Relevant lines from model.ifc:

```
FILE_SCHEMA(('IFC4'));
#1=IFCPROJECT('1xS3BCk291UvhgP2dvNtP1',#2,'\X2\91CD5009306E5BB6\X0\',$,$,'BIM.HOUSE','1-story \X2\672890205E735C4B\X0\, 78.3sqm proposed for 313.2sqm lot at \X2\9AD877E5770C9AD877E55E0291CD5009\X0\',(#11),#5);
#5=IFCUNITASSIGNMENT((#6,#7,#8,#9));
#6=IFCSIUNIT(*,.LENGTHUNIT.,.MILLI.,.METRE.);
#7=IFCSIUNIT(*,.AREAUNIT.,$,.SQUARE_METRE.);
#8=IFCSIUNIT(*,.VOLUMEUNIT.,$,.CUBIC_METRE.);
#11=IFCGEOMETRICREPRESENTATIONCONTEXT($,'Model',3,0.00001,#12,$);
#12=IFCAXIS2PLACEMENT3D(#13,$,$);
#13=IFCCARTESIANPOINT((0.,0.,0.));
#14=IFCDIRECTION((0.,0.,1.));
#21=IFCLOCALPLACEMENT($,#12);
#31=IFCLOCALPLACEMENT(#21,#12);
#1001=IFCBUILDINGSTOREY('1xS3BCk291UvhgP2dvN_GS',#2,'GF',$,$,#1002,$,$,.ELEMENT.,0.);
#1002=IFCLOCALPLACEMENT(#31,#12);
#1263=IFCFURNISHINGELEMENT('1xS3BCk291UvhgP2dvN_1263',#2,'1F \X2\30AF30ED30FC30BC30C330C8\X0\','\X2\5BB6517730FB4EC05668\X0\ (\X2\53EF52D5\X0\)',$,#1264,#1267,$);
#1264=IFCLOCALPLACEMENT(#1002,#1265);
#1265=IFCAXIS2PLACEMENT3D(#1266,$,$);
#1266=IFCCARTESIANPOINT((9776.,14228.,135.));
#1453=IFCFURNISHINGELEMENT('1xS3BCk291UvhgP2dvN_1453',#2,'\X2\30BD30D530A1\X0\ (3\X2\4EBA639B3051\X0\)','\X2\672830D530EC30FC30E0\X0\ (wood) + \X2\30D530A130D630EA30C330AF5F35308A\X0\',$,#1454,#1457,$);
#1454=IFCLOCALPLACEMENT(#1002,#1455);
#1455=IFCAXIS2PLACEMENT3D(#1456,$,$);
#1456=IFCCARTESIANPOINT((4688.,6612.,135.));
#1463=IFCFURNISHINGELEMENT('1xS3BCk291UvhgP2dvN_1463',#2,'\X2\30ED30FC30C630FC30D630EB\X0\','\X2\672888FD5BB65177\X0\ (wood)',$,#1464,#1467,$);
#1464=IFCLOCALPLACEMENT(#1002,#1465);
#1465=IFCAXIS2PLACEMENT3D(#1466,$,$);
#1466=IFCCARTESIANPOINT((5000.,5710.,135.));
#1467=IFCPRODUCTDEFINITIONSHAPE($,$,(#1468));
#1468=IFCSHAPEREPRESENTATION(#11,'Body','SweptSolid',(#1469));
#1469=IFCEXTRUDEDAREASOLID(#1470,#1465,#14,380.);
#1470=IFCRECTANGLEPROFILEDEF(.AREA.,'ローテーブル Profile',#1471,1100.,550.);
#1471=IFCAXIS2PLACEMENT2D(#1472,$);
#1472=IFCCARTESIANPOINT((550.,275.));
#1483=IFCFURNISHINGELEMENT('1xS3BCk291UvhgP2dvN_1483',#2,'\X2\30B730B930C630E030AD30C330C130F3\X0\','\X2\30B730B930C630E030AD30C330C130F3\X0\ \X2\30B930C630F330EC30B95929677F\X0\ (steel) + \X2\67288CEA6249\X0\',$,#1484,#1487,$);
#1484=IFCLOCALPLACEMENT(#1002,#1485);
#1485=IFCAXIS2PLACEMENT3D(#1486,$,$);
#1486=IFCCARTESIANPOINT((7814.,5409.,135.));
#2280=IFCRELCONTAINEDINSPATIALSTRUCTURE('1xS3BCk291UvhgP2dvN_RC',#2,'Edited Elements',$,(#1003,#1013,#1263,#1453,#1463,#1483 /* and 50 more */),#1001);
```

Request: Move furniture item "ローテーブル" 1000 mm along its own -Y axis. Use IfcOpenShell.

```python
import ifcopenshell
import ifcopenshell.api.geometry
import ifcopenshell.util.placement

model = ifcopenshell.open("model.ifc")

item = model.by_guid("1xS3BCk291UvhgP2dvN_1463")
matrix = ifcopenshell.util.placement.get_local_placement(item.ObjectPlacement)
matrix[:3, 3] -= matrix[:3, 1] * 1000.0
ifcopenshell.api.geometry.edit_object_placement(model, product=item, matrix=matrix, is_si=False)

print(ifcopenshell.util.placement.get_local_placement(item.ObjectPlacement).round(3) + 0.0)

model.write("model_edited.ifc")
```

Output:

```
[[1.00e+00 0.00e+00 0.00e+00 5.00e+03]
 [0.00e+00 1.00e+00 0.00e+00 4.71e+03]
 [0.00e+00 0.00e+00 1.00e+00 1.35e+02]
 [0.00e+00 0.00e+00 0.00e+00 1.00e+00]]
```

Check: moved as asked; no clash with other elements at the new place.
